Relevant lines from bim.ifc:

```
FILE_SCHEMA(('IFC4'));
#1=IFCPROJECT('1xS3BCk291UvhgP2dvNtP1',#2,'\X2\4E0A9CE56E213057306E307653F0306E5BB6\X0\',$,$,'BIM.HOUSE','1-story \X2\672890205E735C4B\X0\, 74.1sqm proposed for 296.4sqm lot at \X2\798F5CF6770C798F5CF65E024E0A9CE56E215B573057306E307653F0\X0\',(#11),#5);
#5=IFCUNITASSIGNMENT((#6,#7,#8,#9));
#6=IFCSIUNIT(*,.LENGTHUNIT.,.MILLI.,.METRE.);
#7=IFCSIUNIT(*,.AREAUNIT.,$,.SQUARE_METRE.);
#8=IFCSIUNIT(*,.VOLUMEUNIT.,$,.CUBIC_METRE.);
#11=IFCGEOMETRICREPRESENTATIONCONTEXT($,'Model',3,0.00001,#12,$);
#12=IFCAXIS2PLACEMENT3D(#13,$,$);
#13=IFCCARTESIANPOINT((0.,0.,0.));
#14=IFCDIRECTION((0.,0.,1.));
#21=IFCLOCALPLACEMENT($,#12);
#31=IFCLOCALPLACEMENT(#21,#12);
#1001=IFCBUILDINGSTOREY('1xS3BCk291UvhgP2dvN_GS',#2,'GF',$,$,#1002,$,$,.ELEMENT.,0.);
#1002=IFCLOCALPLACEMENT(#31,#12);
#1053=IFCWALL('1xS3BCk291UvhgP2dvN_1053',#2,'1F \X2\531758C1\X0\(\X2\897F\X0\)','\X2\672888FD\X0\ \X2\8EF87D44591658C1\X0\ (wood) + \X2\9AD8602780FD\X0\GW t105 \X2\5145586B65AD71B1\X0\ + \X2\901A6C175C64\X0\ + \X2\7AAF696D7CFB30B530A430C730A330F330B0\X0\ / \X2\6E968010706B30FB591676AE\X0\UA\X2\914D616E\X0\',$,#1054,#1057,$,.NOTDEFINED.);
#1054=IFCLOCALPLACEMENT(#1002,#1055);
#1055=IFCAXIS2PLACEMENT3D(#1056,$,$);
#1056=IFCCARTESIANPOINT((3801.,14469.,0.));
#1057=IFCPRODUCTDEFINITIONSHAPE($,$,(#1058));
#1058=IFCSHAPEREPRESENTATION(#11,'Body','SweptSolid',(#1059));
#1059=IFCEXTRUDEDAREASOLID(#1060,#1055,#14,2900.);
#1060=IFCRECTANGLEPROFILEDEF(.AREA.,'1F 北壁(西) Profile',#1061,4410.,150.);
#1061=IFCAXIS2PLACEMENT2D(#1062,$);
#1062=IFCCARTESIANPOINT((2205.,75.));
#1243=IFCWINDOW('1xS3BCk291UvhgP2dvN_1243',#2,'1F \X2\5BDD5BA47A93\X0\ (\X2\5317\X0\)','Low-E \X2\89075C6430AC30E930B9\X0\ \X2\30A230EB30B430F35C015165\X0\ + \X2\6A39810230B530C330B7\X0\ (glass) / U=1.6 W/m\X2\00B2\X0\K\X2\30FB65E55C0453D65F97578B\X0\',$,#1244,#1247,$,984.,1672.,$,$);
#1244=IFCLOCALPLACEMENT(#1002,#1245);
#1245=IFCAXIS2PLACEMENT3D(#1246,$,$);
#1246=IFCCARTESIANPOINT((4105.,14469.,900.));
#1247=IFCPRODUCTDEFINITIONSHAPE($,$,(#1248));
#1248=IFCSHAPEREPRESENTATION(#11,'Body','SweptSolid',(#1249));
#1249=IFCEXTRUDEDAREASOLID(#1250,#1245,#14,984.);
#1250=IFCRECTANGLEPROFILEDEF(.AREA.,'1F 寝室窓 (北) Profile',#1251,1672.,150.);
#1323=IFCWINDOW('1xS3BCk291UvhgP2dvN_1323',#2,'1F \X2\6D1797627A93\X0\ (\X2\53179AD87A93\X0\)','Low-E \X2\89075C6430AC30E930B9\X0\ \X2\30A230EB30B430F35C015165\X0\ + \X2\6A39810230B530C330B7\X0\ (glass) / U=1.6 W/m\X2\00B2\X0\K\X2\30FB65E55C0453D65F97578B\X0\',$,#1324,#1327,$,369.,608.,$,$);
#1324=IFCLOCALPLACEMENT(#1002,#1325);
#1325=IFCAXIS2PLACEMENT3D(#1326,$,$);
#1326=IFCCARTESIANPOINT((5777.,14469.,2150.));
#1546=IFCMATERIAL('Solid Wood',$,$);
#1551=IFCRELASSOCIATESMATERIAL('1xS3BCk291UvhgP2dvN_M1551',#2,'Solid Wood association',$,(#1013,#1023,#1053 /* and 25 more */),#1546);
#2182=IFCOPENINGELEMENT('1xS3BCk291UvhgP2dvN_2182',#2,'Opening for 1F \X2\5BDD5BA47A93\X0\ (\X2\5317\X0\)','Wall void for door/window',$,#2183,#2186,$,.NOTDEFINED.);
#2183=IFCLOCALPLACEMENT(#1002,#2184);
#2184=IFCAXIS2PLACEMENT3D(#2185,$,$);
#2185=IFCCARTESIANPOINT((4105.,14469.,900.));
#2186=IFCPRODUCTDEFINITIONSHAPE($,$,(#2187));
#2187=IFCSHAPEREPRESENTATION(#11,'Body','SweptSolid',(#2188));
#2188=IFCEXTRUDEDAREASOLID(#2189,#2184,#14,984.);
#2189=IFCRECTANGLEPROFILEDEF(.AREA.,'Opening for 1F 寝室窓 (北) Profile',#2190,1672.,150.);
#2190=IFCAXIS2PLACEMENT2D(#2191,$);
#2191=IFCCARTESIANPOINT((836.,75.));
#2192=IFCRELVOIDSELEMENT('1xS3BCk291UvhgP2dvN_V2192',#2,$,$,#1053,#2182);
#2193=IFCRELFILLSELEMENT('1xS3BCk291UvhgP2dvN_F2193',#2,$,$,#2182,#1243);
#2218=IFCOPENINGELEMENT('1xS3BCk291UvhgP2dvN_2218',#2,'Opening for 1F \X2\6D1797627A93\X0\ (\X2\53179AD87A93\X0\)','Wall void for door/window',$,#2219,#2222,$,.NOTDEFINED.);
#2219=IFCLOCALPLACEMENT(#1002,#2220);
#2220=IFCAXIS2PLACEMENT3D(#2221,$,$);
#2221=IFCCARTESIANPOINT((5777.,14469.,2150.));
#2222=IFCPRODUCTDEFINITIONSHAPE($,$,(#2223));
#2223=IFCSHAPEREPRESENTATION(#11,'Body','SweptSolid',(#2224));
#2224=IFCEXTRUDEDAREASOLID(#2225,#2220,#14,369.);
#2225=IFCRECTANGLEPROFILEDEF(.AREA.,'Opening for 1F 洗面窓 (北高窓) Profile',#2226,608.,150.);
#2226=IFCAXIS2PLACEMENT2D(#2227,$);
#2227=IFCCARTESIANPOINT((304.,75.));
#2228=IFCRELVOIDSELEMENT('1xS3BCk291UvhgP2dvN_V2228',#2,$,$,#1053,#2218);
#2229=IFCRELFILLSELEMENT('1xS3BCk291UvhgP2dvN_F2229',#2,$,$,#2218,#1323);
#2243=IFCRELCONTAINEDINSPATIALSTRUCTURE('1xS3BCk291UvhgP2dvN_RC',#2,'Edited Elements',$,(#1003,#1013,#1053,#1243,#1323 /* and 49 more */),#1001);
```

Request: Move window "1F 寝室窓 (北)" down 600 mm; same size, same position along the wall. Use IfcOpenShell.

```python
import numpy as np
import ifcopenshell
import ifcopenshell.api.geometry
import ifcopenshell.util.placement
import ifcopenshell.util.unit

model = ifcopenshell.open("bim.ifc")
unit_scale = ifcopenshell.util.unit.calculate_unit_scale(model)

window = model.by_guid("1xS3BCk291UvhgP2dvN_1243")
opening = window.FillsVoids[0].RelatingOpeningElement
dz = -0.6 / unit_scale

shift = np.array([0.0, 0.0, dz])
# The window is not placed relative to its opening, so move both.
for product in (opening, window):
    matrix = ifcopenshell.util.placement.get_local_placement(product.ObjectPlacement)
    matrix[:3, 3] += shift
    ifcopenshell.api.geometry.edit_object_placement(model, product=product, matrix=matrix, is_si=False)

print(f"moved by {dz * unit_scale:+.3f} m")

model.write("bim_updated.ifc")
```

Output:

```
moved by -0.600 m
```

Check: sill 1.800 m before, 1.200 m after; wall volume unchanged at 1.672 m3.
